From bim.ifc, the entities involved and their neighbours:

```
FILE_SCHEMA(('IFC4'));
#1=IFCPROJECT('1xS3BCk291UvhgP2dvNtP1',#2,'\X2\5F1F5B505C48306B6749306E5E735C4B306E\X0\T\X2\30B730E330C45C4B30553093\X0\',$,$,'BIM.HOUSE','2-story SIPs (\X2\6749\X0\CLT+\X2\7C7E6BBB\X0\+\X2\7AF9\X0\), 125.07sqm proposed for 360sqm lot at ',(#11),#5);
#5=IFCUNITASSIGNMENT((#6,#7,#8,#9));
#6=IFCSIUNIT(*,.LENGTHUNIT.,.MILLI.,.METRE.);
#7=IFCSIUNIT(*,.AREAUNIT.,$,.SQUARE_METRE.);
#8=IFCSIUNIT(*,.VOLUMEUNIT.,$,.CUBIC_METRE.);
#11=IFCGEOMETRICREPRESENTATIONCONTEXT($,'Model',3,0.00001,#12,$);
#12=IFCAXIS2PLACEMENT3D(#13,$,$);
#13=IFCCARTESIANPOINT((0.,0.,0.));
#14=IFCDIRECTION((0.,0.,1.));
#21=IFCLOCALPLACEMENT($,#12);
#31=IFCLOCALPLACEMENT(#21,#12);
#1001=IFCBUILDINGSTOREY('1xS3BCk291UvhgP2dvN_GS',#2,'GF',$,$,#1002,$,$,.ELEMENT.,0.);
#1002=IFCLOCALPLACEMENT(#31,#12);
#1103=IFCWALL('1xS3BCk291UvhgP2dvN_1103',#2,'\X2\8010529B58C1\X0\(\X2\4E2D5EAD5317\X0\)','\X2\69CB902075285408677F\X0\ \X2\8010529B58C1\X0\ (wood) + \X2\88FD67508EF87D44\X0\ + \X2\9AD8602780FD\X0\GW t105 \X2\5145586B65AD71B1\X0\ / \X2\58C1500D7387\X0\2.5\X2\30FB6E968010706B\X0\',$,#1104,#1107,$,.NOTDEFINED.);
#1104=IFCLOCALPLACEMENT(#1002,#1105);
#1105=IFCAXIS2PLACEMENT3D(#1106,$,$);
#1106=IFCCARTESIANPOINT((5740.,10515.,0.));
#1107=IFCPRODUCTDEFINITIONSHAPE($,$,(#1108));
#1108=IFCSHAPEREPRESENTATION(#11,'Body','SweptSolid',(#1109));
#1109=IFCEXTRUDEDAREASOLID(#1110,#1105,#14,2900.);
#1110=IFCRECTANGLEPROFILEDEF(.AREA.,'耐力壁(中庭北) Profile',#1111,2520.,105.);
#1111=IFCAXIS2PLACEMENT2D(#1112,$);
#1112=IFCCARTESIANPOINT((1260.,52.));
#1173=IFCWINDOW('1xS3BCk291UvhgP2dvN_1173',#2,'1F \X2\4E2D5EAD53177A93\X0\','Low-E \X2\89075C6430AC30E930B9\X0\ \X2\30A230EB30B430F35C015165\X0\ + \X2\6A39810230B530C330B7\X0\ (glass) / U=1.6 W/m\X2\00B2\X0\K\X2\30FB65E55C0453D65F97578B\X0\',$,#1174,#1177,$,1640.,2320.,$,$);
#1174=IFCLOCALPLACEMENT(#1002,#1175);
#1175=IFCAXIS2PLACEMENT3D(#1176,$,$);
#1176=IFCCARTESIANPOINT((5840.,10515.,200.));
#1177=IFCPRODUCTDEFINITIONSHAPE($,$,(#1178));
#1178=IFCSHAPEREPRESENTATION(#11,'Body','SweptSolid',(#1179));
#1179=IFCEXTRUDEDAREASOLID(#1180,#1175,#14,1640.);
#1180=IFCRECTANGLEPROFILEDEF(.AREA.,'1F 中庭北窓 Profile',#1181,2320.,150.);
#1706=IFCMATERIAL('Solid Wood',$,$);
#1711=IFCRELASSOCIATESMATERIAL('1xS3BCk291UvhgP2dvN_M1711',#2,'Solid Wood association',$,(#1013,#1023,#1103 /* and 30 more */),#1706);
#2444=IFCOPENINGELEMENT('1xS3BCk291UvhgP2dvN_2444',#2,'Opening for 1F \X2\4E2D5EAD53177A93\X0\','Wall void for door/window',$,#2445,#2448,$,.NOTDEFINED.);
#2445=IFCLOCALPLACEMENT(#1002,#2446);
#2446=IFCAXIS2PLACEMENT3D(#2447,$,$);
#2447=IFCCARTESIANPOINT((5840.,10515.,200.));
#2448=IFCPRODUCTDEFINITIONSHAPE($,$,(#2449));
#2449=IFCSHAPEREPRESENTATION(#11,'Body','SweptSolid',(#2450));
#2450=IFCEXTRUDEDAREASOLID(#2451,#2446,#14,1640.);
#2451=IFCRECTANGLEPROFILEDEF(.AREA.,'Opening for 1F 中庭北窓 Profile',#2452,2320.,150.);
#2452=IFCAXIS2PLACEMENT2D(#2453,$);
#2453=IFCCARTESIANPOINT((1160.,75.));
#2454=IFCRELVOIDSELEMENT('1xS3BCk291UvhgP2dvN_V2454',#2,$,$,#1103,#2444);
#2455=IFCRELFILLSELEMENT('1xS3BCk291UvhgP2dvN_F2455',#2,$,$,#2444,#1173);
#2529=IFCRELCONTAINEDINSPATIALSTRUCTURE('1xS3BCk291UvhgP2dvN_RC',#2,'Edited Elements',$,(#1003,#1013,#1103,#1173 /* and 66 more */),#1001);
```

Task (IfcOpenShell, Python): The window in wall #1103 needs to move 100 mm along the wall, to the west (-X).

```python
import ifcopenshell
import ifcopenshell.api.geometry
import ifcopenshell.util.placement

model = ifcopenshell.open("bim.ifc")

window = model.by_id(1173)
opening = window.FillsVoids[0].RelatingOpeningElement
wall = opening.VoidsElements[0].RelatingBuildingElement

wall_matrix = ifcopenshell.util.placement.get_local_placement(wall.ObjectPlacement)
shift = wall_matrix[:3, 0] * -100.0
before = ifcopenshell.util.placement.get_local_placement(window.ObjectPlacement)[:3, 3].copy()

# The window is not placed relative to its opening, so move both.
for product in (opening, window):
    matrix = ifcopenshell.util.placement.get_local_placement(product.ObjectPlacement)
    matrix[:3, 3] += shift
    ifcopenshell.api.geometry.edit_object_placement(model, product=product, matrix=matrix, is_si=False)

after = ifcopenshell.util.placement.get_local_placement(window.ObjectPlacement)[:3, 3]
print("window moved by", (after - before).round(3) + 0.0)

model.write("bim-out.ifc")
```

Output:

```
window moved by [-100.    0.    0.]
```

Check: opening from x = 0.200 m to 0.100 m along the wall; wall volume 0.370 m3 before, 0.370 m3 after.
